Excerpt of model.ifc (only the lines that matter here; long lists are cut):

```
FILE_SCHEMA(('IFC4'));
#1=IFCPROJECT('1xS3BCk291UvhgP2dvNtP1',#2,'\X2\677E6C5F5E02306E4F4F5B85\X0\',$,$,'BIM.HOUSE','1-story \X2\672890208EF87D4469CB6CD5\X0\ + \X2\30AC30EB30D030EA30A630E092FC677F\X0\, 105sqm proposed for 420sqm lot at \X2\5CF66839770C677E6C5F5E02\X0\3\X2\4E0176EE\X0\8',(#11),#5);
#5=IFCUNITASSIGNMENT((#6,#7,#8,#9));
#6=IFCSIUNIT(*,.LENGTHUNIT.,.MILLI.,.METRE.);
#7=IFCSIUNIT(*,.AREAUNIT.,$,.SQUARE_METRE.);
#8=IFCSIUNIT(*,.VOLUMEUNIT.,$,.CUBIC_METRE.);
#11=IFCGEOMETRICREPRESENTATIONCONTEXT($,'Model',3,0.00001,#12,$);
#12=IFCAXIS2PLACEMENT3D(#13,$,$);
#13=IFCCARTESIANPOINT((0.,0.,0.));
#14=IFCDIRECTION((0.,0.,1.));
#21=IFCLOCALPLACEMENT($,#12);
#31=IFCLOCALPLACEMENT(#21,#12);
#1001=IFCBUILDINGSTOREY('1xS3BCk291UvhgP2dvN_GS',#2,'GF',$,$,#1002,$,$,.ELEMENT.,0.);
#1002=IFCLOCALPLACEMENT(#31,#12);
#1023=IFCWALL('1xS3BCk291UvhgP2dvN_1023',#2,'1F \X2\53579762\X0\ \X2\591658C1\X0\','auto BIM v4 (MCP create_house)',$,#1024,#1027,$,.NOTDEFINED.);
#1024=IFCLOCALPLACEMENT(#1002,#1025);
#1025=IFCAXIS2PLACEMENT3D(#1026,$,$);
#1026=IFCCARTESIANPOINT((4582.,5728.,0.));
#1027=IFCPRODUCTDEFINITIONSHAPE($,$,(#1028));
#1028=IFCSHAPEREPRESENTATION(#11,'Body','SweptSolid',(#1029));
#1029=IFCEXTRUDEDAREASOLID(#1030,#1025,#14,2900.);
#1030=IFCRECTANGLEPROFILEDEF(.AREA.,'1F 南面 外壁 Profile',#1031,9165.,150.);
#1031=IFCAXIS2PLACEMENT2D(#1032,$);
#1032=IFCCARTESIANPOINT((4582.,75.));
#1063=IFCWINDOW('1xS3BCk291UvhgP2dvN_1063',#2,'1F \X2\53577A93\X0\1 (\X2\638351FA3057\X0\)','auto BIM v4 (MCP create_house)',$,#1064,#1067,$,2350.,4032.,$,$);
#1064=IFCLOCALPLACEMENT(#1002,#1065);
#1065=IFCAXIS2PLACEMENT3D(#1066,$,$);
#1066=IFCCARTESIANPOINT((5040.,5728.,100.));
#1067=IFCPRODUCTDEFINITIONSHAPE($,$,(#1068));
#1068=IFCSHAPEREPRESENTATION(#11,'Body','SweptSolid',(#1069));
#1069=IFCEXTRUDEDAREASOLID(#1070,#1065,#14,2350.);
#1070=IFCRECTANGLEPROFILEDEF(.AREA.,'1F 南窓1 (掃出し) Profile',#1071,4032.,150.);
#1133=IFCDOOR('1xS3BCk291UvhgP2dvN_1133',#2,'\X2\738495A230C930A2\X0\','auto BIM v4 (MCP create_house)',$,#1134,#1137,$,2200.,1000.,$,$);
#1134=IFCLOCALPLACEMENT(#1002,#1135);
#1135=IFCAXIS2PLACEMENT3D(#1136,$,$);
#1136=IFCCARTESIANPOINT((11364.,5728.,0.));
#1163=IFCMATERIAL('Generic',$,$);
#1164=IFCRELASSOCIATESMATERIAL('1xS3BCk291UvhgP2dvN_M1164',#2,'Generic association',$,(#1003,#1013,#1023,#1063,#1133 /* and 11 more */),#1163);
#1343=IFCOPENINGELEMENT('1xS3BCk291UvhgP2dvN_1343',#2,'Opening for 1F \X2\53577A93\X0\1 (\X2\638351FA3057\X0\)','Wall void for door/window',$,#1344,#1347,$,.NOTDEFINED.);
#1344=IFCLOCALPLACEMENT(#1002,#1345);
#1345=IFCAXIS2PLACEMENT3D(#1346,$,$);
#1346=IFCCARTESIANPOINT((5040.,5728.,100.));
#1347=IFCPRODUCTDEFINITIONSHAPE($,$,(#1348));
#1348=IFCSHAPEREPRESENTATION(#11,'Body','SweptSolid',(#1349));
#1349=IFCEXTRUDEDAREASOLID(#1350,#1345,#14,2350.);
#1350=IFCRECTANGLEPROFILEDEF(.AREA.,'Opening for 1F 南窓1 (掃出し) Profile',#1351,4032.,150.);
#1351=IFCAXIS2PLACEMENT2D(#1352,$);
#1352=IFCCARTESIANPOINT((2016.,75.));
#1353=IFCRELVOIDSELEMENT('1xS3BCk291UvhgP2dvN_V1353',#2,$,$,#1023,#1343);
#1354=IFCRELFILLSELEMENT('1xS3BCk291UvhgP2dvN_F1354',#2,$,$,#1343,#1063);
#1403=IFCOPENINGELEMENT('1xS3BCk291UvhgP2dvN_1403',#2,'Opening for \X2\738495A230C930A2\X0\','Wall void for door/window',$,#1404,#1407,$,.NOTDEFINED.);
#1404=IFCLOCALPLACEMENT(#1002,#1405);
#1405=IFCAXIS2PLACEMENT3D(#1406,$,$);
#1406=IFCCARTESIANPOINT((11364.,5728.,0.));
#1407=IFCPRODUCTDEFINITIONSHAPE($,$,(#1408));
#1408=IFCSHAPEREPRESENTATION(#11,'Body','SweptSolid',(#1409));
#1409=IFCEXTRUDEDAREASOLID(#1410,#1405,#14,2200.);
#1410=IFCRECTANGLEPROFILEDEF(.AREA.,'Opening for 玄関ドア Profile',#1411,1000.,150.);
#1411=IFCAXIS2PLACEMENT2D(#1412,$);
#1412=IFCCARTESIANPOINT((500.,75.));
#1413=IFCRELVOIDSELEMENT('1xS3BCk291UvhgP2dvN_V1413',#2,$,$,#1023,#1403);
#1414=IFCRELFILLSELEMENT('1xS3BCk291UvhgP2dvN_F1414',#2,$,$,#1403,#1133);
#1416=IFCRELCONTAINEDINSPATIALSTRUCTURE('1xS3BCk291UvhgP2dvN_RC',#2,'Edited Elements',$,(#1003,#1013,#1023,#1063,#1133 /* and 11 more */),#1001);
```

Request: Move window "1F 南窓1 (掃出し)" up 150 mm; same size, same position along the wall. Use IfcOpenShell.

```python
import numpy as np
import ifcopenshell
import ifcopenshell.api.geometry
import ifcopenshell.util.placement
import ifcopenshell.util.unit

model = ifcopenshell.open("model.ifc")
unit_scale = ifcopenshell.util.unit.calculate_unit_scale(model)

window = model.by_id(1063)
opening = window.FillsVoids[0].RelatingOpeningElement
dz = 150.0

shift = np.array([0.0, 0.0, dz])
# The window is not placed relative to its opening, so move both.
for product in (opening, window):
    matrix = ifcopenshell.util.placement.get_local_placement(product.ObjectPlacement)
    matrix[:3, 3] += shift
    ifcopenshell.api.geometry.edit_object_placement(model, product=product, matrix=matrix, is_si=False)

print(f"moved by {dz * unit_scale:+.3f} m")

model.write("model_rev.ifc")
```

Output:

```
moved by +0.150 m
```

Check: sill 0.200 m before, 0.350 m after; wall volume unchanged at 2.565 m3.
